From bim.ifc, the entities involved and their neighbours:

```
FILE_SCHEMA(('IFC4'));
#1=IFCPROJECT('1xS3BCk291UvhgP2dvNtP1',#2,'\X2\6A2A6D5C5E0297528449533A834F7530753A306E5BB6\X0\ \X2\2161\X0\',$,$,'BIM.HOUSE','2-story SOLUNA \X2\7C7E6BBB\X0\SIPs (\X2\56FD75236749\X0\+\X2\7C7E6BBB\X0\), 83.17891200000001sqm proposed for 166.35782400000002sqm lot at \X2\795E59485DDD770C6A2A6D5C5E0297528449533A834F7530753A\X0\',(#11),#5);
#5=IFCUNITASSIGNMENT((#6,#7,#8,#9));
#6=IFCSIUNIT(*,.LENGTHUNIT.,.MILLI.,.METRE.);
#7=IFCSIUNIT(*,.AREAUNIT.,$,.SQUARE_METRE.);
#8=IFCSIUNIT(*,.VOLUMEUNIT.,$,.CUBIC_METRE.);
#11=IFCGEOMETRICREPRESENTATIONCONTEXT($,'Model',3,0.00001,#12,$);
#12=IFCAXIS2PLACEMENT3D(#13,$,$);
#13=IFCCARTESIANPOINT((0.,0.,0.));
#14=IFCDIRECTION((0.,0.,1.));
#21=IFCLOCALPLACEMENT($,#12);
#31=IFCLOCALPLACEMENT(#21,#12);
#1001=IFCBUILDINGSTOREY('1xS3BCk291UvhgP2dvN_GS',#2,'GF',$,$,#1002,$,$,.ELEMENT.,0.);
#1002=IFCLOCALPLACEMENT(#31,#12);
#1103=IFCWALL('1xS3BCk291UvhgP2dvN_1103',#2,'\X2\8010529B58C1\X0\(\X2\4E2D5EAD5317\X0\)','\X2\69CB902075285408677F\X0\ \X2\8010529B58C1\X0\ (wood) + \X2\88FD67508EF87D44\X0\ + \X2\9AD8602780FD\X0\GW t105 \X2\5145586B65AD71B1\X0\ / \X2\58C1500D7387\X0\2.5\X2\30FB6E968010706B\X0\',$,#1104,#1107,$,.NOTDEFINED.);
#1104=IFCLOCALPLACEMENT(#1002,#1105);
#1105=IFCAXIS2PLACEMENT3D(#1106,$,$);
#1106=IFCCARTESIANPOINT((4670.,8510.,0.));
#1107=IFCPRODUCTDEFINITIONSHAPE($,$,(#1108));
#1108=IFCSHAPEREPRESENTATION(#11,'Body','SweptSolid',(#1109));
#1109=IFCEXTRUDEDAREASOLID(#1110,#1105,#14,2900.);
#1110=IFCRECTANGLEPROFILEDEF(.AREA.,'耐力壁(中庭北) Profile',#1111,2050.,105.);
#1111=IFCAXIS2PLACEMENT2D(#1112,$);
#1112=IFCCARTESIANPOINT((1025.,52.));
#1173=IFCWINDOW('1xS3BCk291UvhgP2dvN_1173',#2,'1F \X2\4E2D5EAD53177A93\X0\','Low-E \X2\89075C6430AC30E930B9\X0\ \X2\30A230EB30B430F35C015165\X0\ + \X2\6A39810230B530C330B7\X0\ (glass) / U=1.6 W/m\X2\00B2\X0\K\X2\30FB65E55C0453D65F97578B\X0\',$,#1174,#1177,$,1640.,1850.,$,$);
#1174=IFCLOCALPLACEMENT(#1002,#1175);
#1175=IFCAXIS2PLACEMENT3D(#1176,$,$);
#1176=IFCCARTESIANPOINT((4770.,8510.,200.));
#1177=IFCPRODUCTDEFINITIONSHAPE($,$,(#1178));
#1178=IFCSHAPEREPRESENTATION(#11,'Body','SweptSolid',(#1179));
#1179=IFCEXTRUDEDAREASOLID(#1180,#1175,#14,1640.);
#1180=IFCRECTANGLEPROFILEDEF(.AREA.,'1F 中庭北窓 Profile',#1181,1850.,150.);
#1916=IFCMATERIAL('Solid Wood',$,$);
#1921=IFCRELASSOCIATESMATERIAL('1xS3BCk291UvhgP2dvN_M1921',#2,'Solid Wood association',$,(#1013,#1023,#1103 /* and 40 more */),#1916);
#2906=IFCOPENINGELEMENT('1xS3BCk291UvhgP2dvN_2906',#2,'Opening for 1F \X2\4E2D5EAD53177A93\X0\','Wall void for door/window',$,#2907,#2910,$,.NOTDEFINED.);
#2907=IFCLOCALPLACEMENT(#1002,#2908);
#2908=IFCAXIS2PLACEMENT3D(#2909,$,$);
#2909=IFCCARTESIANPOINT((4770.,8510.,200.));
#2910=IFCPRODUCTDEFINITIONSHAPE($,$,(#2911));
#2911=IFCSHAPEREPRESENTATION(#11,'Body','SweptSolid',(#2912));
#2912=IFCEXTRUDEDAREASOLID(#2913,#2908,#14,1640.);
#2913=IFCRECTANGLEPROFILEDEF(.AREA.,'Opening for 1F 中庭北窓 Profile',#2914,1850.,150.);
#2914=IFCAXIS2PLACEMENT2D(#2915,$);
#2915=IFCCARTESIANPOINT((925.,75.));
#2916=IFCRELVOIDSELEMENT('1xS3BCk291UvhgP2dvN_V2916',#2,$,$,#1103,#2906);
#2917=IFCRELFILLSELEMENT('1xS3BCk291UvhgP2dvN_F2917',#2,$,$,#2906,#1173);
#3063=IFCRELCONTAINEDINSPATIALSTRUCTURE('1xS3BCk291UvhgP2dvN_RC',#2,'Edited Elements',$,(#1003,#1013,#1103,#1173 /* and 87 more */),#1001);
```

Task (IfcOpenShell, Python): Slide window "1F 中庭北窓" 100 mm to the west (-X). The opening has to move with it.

```python
import ifcopenshell
import ifcopenshell.api.geometry
import ifcopenshell.util.placement
import ifcopenshell.util.unit

model = ifcopenshell.open("bim.ifc")
unit_scale = ifcopenshell.util.unit.calculate_unit_scale(model)

window = model.by_guid("1xS3BCk291UvhgP2dvN_1173")
opening = window.FillsVoids[0].RelatingOpeningElement
wall = opening.VoidsElements[0].RelatingBuildingElement

wall_matrix = ifcopenshell.util.placement.get_local_placement(wall.ObjectPlacement)
shift = wall_matrix[:3, 0] * -0.1 / unit_scale
before = ifcopenshell.util.placement.get_local_placement(window.ObjectPlacement)[:3, 3].copy()

# The window is not placed relative to its opening, so move both.
for product in (opening, window):
    matrix = ifcopenshell.util.placement.get_local_placement(product.ObjectPlacement)
    matrix[:3, 3] += shift
    ifcopenshell.api.geometry.edit_object_placement(model, product=product, matrix=matrix, is_si=False)

after = ifcopenshell.util.placement.get_local_placement(window.ObjectPlacement)[:3, 3]
print("window moved by", (after - before).round(3) + 0.0)

model.write("bim_updated.ifc")
```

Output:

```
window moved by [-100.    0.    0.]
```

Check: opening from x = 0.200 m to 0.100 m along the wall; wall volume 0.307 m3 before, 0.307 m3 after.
